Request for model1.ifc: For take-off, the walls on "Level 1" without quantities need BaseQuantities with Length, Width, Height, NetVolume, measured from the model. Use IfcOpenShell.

First a look at what the model holds.

```python
import ifcopenshell
import ifcopenshell.util.element
import ifcopenshell.util.unit

model = ifcopenshell.open("model1.ifc")
print(model.schema)
for unit_type in ("LENGTHUNIT", "AREAUNIT", "VOLUMEUNIT"):
    print(unit_type, ifcopenshell.util.unit.calculate_unit_scale(model, unit_type))
storey = next(s for s in model.by_type("IfcBuildingStorey") if s.Name == "Level 1")
walls = [e for e in ifcopenshell.util.element.get_decomposition(storey) if e.is_a("IfcWall")]
for e in sorted(walls, key=lambda e: e.id()):
    print(e.id(), e.is_a(), e.Name, list(ifcopenshell.util.element.get_psets(e, qtos_only=True)), sep=" | ")
```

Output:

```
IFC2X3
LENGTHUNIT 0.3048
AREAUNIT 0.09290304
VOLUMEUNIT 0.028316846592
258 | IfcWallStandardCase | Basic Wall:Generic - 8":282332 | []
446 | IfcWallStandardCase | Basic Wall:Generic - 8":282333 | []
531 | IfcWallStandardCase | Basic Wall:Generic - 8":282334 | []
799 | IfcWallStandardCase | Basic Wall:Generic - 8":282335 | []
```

```python
import ifcopenshell
import ifcopenshell.api.pset
import ifcopenshell.geom
import ifcopenshell.util.element
import ifcopenshell.util.shape
import ifcopenshell.util.unit

model = ifcopenshell.open("model1.ifc")
unit_scale = ifcopenshell.util.unit.calculate_unit_scale(model)
volume_scale = ifcopenshell.util.unit.calculate_unit_scale(model, "VOLUMEUNIT")
settings = ifcopenshell.geom.settings()

storey = next(s for s in model.by_type("IfcBuildingStorey") if s.Name == "Level 1")
walls = [e for e in ifcopenshell.util.element.get_decomposition(storey) if e.is_a("IfcWall")]

for e in sorted(walls, key=lambda e: e.id()):
    if ifcopenshell.util.element.get_psets(e, qtos_only=True, should_inherit=False):
        continue
    # Geometry comes back in metres, in the element's own axes.
    shape = ifcopenshell.geom.create_shape(settings, e)
    values = {
        "Length": ifcopenshell.util.shape.get_x(shape.geometry) / unit_scale,
        "Width": ifcopenshell.util.shape.get_y(shape.geometry) / unit_scale,
        "Height": ifcopenshell.util.shape.get_z(shape.geometry) / unit_scale,
        "NetVolume": ifcopenshell.util.shape.get_volume(shape.geometry) / volume_scale,
    }
    qto = ifcopenshell.api.pset.add_qto(model, product=e, name="BaseQuantities")
    ifcopenshell.api.pset.edit_qto(model, qto=qto, properties=values)
    print(e.id(), {k: round(v, 3) for k, v in values.items()})

model.write("model1-out.ifc")
```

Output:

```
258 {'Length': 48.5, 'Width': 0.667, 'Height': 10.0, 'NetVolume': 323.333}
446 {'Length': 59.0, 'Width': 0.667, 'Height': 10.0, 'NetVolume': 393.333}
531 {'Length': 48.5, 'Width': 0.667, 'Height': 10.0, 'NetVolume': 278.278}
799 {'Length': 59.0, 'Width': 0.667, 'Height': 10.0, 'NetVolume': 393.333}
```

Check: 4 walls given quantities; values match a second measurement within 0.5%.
